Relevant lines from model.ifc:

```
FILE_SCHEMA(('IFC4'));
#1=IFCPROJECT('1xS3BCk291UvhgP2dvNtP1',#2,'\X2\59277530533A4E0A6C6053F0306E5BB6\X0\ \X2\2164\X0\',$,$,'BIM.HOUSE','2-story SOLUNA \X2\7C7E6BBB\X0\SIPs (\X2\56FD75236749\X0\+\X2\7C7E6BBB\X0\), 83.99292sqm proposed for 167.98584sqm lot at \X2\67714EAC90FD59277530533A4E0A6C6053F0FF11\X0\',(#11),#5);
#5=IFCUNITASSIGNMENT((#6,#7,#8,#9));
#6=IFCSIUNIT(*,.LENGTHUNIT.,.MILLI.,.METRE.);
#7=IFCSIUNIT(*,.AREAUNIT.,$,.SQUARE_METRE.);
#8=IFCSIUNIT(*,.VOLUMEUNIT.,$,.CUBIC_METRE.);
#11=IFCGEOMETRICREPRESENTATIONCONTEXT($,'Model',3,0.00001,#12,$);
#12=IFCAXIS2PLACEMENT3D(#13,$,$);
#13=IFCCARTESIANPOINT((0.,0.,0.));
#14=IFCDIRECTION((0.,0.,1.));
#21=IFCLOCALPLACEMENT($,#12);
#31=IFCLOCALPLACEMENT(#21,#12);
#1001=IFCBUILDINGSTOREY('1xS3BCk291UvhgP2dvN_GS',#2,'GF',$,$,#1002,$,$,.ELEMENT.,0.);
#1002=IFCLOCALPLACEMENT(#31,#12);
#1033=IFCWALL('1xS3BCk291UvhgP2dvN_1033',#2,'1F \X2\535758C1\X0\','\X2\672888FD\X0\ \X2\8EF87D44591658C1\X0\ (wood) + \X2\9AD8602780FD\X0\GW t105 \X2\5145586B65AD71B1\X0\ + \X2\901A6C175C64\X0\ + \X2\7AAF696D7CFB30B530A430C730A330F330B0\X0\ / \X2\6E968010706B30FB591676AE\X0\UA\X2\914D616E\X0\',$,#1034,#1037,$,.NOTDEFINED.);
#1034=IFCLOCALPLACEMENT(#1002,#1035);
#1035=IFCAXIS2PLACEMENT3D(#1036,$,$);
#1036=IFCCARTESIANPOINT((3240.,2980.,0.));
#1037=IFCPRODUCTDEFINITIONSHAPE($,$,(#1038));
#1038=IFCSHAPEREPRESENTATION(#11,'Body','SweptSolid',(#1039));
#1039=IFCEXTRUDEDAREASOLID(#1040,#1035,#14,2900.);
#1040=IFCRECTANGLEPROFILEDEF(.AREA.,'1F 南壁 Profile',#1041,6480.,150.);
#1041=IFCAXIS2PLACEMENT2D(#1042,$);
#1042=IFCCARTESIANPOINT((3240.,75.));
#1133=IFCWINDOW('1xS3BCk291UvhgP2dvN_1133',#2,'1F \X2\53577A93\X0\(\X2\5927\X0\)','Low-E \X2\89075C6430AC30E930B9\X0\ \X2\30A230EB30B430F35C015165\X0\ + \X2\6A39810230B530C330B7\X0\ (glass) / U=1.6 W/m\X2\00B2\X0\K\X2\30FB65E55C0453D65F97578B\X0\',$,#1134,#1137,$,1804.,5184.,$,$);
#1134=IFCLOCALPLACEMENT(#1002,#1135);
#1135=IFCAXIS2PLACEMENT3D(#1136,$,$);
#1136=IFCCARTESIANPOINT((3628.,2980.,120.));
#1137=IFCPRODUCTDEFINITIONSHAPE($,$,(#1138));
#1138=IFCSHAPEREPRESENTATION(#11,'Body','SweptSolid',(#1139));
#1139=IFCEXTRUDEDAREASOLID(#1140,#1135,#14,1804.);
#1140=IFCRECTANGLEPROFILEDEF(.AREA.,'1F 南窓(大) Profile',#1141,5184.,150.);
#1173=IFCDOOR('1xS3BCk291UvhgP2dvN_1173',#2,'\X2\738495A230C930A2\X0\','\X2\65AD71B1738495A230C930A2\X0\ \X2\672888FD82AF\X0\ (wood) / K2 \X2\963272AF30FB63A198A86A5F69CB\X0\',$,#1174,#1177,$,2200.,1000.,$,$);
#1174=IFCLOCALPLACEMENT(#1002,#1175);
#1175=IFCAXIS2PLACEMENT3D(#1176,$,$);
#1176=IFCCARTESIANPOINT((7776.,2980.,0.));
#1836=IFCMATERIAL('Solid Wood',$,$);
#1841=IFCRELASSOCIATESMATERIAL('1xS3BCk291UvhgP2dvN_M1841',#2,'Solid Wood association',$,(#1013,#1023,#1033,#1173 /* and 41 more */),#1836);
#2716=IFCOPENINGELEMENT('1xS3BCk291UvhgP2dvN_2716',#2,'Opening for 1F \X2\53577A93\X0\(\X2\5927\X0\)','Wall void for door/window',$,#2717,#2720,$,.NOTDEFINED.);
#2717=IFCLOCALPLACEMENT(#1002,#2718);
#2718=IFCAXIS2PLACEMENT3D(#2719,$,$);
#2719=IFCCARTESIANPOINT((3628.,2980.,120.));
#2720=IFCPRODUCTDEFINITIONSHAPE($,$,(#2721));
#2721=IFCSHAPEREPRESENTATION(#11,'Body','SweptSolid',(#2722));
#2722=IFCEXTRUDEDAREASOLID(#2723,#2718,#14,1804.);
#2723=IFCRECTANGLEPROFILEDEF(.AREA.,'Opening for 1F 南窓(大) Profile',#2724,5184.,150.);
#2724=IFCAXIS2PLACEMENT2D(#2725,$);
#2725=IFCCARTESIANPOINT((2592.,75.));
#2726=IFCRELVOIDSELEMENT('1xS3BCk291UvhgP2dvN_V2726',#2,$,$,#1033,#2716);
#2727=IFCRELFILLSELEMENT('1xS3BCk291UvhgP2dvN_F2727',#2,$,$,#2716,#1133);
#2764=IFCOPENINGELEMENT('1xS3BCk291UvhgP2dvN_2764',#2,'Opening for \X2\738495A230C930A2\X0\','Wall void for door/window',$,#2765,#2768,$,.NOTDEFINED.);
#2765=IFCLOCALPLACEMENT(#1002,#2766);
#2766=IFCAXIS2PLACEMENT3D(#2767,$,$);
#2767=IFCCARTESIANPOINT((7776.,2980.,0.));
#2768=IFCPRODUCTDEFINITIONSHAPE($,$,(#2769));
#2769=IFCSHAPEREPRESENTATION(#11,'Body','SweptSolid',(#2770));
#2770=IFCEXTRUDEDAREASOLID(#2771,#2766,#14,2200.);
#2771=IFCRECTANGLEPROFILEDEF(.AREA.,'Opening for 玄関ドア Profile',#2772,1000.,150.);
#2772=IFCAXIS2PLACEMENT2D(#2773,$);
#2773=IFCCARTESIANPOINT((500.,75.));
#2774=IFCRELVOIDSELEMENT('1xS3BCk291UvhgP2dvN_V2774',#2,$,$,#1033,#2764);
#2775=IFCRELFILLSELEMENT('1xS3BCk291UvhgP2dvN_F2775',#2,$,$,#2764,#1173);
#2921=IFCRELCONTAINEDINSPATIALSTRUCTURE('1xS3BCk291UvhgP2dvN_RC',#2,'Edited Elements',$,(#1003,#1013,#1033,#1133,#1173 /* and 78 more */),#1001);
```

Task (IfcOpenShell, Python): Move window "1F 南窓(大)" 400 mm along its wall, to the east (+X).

```python
import ifcopenshell
import ifcopenshell.api.geometry
import ifcopenshell.util.placement

model = ifcopenshell.open("model.ifc")

window = model.by_id(1133)
opening = window.FillsVoids[0].RelatingOpeningElement
wall = opening.VoidsElements[0].RelatingBuildingElement

wall_matrix = ifcopenshell.util.placement.get_local_placement(wall.ObjectPlacement)
shift = wall_matrix[:3, 0] * 400.0
before = ifcopenshell.util.placement.get_local_placement(window.ObjectPlacement)[:3, 3].copy()

# The window is not placed relative to its opening, so move both.
for product in (opening, window):
    matrix = ifcopenshell.util.placement.get_local_placement(product.ObjectPlacement)
    matrix[:3, 3] += shift
    ifcopenshell.api.geometry.edit_object_placement(model, product=product, matrix=matrix, is_si=False)

after = ifcopenshell.util.placement.get_local_placement(window.ObjectPlacement)[:3, 3]
print("window moved by", (after - before).round(3) + 0.0)

model.write("model_edited.ifc")
```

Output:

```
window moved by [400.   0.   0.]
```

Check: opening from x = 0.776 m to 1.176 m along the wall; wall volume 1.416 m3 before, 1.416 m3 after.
